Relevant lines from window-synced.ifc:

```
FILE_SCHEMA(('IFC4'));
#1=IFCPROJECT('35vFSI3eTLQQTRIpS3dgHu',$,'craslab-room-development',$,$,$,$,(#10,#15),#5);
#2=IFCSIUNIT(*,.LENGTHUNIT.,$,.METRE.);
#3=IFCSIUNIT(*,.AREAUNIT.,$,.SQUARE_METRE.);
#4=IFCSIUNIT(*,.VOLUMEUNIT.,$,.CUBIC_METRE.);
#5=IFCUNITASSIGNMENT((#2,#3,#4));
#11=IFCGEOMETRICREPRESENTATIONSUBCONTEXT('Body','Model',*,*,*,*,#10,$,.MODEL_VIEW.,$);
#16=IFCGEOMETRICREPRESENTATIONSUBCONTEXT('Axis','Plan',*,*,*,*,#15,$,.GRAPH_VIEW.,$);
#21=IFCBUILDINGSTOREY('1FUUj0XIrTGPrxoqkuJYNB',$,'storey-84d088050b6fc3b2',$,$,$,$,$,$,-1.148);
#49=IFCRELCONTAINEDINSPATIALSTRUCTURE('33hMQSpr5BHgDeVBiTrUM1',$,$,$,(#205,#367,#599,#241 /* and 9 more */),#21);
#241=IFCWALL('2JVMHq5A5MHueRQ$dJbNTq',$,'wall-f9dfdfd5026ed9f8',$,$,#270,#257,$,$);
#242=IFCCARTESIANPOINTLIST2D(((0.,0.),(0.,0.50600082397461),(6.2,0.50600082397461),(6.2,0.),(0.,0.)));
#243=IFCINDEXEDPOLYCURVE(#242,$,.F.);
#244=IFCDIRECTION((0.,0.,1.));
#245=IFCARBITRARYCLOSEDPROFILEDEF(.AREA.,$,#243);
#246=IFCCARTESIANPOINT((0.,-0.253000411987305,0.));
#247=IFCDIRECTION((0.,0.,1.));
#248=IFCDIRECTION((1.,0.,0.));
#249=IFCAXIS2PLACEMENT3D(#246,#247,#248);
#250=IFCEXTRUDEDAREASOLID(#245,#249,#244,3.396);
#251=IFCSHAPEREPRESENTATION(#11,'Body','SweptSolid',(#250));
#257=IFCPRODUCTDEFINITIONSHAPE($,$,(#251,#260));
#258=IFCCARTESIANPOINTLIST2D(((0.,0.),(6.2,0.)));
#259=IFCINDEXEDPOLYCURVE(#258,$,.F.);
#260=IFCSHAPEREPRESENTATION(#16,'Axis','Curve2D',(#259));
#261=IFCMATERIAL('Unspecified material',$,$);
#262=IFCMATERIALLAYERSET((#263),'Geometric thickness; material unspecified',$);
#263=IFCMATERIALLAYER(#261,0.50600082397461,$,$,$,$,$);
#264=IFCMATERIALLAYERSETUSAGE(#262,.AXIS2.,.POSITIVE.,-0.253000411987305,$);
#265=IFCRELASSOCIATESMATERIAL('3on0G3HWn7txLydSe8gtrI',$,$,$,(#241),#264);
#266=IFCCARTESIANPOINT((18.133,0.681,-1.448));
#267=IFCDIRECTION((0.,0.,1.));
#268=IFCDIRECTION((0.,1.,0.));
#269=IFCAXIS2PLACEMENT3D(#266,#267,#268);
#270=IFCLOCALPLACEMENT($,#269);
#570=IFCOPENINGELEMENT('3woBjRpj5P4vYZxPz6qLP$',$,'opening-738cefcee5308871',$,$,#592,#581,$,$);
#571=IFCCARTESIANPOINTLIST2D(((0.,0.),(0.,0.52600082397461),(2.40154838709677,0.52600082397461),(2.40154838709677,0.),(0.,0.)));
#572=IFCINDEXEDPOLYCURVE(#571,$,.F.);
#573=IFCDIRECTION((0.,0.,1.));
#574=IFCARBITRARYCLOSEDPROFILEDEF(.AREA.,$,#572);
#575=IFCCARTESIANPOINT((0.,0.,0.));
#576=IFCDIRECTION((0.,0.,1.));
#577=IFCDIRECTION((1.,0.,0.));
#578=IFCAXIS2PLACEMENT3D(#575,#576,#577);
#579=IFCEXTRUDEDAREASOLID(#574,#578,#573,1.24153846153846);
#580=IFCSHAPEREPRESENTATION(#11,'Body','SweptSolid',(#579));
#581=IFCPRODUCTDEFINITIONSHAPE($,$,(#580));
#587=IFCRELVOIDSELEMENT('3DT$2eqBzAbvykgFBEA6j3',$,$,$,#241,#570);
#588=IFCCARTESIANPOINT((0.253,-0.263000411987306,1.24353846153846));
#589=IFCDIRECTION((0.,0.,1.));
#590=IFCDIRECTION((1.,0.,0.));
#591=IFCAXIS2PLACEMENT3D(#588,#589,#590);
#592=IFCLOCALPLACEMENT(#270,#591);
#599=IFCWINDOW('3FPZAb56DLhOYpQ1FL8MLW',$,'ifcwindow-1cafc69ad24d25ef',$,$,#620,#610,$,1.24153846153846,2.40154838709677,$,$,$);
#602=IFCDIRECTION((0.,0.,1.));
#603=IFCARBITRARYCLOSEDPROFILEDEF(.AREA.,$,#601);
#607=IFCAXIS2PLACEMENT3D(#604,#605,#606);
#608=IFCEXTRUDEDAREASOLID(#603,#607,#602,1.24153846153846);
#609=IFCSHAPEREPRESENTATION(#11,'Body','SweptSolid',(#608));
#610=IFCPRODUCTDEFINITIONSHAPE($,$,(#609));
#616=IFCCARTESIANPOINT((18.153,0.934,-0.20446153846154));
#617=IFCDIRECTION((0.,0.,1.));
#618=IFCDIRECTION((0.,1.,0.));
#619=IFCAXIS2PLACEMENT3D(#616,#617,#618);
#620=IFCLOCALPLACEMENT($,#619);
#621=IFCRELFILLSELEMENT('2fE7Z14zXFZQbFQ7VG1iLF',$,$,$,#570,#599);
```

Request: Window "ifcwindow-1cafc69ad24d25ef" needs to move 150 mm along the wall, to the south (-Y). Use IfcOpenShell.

```python
import ifcopenshell
import ifcopenshell.api.geometry
import ifcopenshell.util.placement
import ifcopenshell.util.unit

model = ifcopenshell.open("window-synced.ifc")
unit_scale = ifcopenshell.util.unit.calculate_unit_scale(model)

window = model.by_guid("3FPZAb56DLhOYpQ1FL8MLW")
opening = window.FillsVoids[0].RelatingOpeningElement
wall = opening.VoidsElements[0].RelatingBuildingElement

wall_matrix = ifcopenshell.util.placement.get_local_placement(wall.ObjectPlacement)
shift = wall_matrix[:3, 0] * -0.15 / unit_scale
before = ifcopenshell.util.placement.get_local_placement(window.ObjectPlacement)[:3, 3].copy()

# The window is not placed relative to its opening, so move both.
for product in (opening, window):
    matrix = ifcopenshell.util.placement.get_local_placement(product.ObjectPlacement)
    matrix[:3, 3] += shift
    ifcopenshell.api.geometry.edit_object_placement(model, product=product, matrix=matrix, is_si=False)

after = ifcopenshell.util.placement.get_local_placement(window.ObjectPlacement)[:3, 3]
print("window moved by", (after - before).round(3) + 0.0)

model.write("window-synced_rev.ifc")
```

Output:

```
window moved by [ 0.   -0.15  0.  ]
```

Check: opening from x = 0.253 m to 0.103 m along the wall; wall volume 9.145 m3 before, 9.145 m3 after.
